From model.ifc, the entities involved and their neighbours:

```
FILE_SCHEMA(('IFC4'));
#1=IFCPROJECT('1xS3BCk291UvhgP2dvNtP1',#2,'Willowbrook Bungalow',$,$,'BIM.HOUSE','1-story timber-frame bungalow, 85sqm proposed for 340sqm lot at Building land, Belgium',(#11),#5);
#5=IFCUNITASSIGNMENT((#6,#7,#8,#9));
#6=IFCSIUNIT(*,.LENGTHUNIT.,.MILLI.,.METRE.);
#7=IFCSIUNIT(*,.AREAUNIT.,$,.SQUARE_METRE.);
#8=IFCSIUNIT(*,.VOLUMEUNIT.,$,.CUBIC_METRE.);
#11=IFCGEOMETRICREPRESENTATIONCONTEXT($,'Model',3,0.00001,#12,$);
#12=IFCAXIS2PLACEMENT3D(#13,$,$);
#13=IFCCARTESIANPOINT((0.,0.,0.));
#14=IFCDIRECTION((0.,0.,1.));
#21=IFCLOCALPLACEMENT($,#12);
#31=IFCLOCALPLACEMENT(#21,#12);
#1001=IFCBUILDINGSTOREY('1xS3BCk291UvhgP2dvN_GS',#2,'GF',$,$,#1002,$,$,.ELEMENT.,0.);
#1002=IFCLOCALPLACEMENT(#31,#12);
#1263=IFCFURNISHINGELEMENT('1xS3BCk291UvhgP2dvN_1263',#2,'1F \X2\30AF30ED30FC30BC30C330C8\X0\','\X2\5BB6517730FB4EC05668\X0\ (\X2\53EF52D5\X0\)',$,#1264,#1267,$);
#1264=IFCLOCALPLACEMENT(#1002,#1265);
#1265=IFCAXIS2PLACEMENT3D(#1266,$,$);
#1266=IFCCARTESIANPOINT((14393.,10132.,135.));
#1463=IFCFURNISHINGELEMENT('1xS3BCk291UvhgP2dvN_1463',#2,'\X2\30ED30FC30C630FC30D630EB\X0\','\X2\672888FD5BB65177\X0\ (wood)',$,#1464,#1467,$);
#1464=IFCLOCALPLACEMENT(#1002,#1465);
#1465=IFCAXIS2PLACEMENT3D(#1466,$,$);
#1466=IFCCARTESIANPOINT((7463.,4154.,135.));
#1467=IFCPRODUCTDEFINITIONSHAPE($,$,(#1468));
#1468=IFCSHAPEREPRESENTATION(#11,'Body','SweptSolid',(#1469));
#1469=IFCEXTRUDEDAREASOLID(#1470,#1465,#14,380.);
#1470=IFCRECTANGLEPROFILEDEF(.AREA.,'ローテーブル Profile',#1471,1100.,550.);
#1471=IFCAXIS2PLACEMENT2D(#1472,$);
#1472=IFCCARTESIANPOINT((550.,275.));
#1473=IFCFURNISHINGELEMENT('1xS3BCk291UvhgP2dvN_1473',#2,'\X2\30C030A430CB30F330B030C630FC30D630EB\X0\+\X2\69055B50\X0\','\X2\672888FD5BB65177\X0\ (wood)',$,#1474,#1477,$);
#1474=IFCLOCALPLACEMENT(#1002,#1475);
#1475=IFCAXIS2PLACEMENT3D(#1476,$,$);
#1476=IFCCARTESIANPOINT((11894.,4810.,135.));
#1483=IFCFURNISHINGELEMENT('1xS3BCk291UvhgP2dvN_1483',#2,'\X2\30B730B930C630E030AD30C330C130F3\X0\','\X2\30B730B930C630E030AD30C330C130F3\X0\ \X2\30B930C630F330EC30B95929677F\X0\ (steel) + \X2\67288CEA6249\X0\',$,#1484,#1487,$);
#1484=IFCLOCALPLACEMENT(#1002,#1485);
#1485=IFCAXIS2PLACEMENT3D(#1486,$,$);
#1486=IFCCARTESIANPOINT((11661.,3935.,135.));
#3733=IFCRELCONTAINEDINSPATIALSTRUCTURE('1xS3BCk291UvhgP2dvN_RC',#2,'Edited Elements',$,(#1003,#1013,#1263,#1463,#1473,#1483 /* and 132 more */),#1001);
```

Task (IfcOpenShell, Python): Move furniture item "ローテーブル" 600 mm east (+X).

```python
import ifcopenshell
import ifcopenshell.api.geometry
import ifcopenshell.util.placement
import ifcopenshell.util.unit

model = ifcopenshell.open("model.ifc")
unit_scale = ifcopenshell.util.unit.calculate_unit_scale(model)

item = model.by_guid("1xS3BCk291UvhgP2dvN_1463")
matrix = ifcopenshell.util.placement.get_local_placement(item.ObjectPlacement)
matrix[0, 3] += 0.6 / unit_scale
ifcopenshell.api.geometry.edit_object_placement(model, product=item, matrix=matrix, is_si=False)

print(ifcopenshell.util.placement.get_local_placement(item.ObjectPlacement).round(3) + 0.0)

model.write("model_edited.ifc")
```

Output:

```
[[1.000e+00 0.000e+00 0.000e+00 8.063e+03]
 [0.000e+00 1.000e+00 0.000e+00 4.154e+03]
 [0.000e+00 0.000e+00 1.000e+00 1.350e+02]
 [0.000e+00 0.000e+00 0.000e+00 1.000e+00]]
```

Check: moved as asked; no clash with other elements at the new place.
